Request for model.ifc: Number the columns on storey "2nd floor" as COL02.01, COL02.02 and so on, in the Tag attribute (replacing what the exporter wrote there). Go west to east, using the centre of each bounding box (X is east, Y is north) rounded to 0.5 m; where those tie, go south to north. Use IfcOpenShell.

First a look at what the model holds.

```python
import ifcopenshell
import ifcopenshell.util.element
import ifcopenshell.util.placement

model = ifcopenshell.open("model.ifc")
print(model.schema)
storey = next(s for s in model.by_type("IfcBuildingStorey") if s.Name == "2nd floor")
columns = [e for e in ifcopenshell.util.element.get_decomposition(storey) if e.is_a("IfcColumn")]
for e in sorted(columns, key=lambda e: e.id()):
    origin = ifcopenshell.util.placement.get_local_placement(e.ObjectPlacement)[:3, 3]
    print(e.id(), e.Tag, e.Name, origin.round(2) + 0.0, sep=" | ")
```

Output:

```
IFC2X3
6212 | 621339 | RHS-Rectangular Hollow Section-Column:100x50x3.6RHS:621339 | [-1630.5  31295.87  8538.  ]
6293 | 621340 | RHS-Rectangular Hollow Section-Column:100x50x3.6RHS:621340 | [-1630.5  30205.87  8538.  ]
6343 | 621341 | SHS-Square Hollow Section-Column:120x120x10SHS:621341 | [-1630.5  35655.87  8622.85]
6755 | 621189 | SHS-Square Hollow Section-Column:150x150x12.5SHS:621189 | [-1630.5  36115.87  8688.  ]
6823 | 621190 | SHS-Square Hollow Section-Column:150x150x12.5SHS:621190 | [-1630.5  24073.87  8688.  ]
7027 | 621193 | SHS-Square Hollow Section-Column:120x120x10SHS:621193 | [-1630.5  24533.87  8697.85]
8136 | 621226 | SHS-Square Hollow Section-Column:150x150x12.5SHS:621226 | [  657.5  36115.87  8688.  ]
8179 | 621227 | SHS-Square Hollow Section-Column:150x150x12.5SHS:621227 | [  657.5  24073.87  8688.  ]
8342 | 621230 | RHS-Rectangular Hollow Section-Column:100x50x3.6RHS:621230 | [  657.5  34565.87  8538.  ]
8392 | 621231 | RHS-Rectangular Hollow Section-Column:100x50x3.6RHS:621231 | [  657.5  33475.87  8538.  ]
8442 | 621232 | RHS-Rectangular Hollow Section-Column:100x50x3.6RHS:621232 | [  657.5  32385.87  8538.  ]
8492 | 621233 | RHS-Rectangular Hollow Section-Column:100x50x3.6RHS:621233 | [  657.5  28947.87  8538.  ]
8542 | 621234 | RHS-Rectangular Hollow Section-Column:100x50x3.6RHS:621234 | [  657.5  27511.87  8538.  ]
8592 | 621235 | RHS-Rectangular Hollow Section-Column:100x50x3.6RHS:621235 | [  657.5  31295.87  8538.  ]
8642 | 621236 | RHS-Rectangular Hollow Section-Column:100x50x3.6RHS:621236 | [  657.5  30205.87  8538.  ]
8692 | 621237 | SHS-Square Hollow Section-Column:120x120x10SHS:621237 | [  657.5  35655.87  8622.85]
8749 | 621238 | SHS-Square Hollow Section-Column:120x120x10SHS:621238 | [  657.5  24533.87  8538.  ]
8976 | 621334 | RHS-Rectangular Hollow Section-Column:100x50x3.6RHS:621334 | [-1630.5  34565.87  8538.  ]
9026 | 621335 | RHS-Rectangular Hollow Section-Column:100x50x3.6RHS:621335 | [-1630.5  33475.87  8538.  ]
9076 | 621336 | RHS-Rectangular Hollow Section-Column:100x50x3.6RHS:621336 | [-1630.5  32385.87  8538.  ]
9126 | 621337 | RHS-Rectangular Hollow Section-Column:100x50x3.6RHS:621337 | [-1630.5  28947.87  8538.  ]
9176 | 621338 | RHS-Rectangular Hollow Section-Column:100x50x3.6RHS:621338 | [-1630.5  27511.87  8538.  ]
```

```python
import ifcopenshell
import ifcopenshell.geom
import ifcopenshell.util.element
import ifcopenshell.util.shape

model = ifcopenshell.open("model.ifc")
settings = ifcopenshell.geom.settings()
settings.set("use-world-coords", True)


def centre(element):
    shape = ifcopenshell.geom.create_shape(settings, element)
    return ifcopenshell.util.shape.get_bbox_centroid(shape.geometry)


storey = next(s for s in model.by_type("IfcBuildingStorey") if s.Name == "2nd floor")
columns = [e for e in ifcopenshell.util.element.get_decomposition(storey) if e.is_a("IfcColumn")]

# Insertion points can sit at a corner or the storey origin, so sort by the geometry (in metres).
centres = {e: centre(e) for e in columns}
columns.sort(key=lambda e: (round(centres[e][0] / 0.5), centres[e][1]))

for i, e in enumerate(columns, start=1):
    number = f"COL02.{i:02d}"
    e.Tag = number
    print(e.id(), number)

model.write("model_edited.ifc")
```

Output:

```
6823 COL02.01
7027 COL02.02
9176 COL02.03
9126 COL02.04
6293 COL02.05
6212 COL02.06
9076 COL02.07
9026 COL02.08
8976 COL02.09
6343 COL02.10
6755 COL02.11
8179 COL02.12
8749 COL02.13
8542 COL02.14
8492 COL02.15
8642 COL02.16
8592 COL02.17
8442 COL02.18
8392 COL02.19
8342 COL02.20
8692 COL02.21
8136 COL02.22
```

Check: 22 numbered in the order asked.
